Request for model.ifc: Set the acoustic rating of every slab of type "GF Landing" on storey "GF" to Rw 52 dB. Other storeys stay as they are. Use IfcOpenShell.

First a look at what the model holds.

```python
import ifcopenshell
import ifcopenshell.util.element

model = ifcopenshell.open("model.ifc")
print(model.schema)
storey = next(s for s in model.by_type("IfcBuildingStorey") if s.Name == "GF")
slabs = [e for e in ifcopenshell.util.element.get_decomposition(storey) if e.is_a("IfcSlab")]
seen = {}
for e in slabs:
    element_type = ifcopenshell.util.element.get_type(e)
    key = (element_type.Name if element_type != e and element_type else None, ifcopenshell.util.element.get_pset(e, "Pset_SlabCommon", "AcousticRating"))
    seen[key] = seen.get(key, 0) + 1
for (name, value), count in sorted(seen.items(), key=str):
    print(count, "x", name, "|", value)
```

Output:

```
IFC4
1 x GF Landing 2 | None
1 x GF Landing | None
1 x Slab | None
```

```python
import ifcopenshell
import ifcopenshell.api.pset
import ifcopenshell.util.element

model = ifcopenshell.open("model.ifc")

storey = next(s for s in model.by_type("IfcBuildingStorey") if s.Name == "GF")
slabs = [e for e in ifcopenshell.util.element.get_decomposition(storey) if e.is_a("IfcSlab")]

count = 0
for e in slabs:
    element_type = ifcopenshell.util.element.get_type(e)
    if element_type in (None, e) or element_type.Name != "GF Landing":
        continue
    # add_pset returns the element's existing set when there is one.
    pset = ifcopenshell.api.pset.add_pset(model, product=e, name="Pset_SlabCommon")
    ifcopenshell.api.pset.edit_pset(model, pset=pset, properties={"AcousticRating": "Rw 52 dB"})
    count += 1

print(count, "slabs updated")

model.write("model_updated.ifc")
```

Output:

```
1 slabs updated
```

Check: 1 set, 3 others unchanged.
